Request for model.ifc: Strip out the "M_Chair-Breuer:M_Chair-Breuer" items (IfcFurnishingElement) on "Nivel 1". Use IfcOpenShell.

First a look at what the model holds.

```python
import ifcopenshell
import ifcopenshell.util.element

model = ifcopenshell.open("model.ifc")
print(model.schema)
storey = next(s for s in model.by_type("IfcBuildingStorey") if s.Name == "Nivel 1")
furniture = [e for e in ifcopenshell.util.element.get_decomposition(storey) if e.is_a("IfcFurnishingElement")]
seen = {}
for e in furniture:
    element_type = ifcopenshell.util.element.get_type(e)
    name = element_type.Name if element_type not in (None, e) else None
    seen[name] = seen.get(name, 0) + 1
for name, count in sorted(seen.items(), key=str):
    print(count, "x", name)
```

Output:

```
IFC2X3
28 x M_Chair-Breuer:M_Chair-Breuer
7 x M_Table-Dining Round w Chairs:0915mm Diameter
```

```python
import ifcopenshell
import ifcopenshell.api.root
import ifcopenshell.util.element

model = ifcopenshell.open("model.ifc")

storey = next(s for s in model.by_type("IfcBuildingStorey") if s.Name == "Nivel 1")
furniture = [e for e in ifcopenshell.util.element.get_decomposition(storey) if e.is_a("IfcFurnishingElement")]
targets = [e for e in furniture if (t := ifcopenshell.util.element.get_type(e)) not in (None, e) and t.Name == "M_Chair-Breuer:M_Chair-Breuer"]

for e in targets:
    ifcopenshell.api.root.remove_product(model, product=e)
print(len(targets), "removed")

model.write("model_v2.ifc")
```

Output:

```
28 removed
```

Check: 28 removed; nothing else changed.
